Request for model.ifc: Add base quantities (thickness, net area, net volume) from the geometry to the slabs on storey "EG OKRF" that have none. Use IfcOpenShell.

First a look at what the model holds.

```python
import ifcopenshell
import ifcopenshell.util.element
import ifcopenshell.util.unit

model = ifcopenshell.open("model.ifc")
print(model.schema)
for unit_type in ("LENGTHUNIT", "AREAUNIT", "VOLUMEUNIT"):
    print(unit_type, ifcopenshell.util.unit.calculate_unit_scale(model, unit_type))
storey = next(s for s in model.by_type("IfcBuildingStorey") if s.Name == "EG OKRF")
slabs = [e for e in ifcopenshell.util.element.get_decomposition(storey) if e.is_a("IfcSlab")]
for e in sorted(slabs, key=lambda e: e.id()):
    print(e.id(), e.is_a(), e.Name, list(ifcopenshell.util.element.get_psets(e, qtos_only=True)), sep=" | ")
```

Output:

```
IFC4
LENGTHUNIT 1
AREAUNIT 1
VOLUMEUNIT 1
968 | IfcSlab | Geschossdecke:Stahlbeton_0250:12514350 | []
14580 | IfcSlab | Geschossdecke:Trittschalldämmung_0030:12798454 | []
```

```python
import ifcopenshell
import ifcopenshell.api.pset
import ifcopenshell.geom
import ifcopenshell.util.element
import ifcopenshell.util.shape
import ifcopenshell.util.unit

model = ifcopenshell.open("model.ifc")
unit_scale = ifcopenshell.util.unit.calculate_unit_scale(model)
area_scale = ifcopenshell.util.unit.calculate_unit_scale(model, "AREAUNIT")
volume_scale = ifcopenshell.util.unit.calculate_unit_scale(model, "VOLUMEUNIT")
settings = ifcopenshell.geom.settings()

storey = next(s for s in model.by_type("IfcBuildingStorey") if s.Name == "EG OKRF")
slabs = [e for e in ifcopenshell.util.element.get_decomposition(storey) if e.is_a("IfcSlab")]

for e in sorted(slabs, key=lambda e: e.id()):
    if ifcopenshell.util.element.get_psets(e, qtos_only=True, should_inherit=False):
        continue
    # Geometry comes back in metres, in the element's own axes.
    shape = ifcopenshell.geom.create_shape(settings, e)
    values = {
        "Width": ifcopenshell.util.shape.get_z(shape.geometry) / unit_scale,
        "NetArea": ifcopenshell.util.shape.get_footprint_area(shape.geometry) / area_scale,
        "NetVolume": ifcopenshell.util.shape.get_volume(shape.geometry) / volume_scale,
    }
    qto = ifcopenshell.api.pset.add_qto(model, product=e, name="Qto_SlabBaseQuantities")
    ifcopenshell.api.pset.edit_qto(model, qto=qto, properties=values)
    print(e.id(), {k: round(v, 3) for k, v in values.items()})

model.write("model-out.ifc")
```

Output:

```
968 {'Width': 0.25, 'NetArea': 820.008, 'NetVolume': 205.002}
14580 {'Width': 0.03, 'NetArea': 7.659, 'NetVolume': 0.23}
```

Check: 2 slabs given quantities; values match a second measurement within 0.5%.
